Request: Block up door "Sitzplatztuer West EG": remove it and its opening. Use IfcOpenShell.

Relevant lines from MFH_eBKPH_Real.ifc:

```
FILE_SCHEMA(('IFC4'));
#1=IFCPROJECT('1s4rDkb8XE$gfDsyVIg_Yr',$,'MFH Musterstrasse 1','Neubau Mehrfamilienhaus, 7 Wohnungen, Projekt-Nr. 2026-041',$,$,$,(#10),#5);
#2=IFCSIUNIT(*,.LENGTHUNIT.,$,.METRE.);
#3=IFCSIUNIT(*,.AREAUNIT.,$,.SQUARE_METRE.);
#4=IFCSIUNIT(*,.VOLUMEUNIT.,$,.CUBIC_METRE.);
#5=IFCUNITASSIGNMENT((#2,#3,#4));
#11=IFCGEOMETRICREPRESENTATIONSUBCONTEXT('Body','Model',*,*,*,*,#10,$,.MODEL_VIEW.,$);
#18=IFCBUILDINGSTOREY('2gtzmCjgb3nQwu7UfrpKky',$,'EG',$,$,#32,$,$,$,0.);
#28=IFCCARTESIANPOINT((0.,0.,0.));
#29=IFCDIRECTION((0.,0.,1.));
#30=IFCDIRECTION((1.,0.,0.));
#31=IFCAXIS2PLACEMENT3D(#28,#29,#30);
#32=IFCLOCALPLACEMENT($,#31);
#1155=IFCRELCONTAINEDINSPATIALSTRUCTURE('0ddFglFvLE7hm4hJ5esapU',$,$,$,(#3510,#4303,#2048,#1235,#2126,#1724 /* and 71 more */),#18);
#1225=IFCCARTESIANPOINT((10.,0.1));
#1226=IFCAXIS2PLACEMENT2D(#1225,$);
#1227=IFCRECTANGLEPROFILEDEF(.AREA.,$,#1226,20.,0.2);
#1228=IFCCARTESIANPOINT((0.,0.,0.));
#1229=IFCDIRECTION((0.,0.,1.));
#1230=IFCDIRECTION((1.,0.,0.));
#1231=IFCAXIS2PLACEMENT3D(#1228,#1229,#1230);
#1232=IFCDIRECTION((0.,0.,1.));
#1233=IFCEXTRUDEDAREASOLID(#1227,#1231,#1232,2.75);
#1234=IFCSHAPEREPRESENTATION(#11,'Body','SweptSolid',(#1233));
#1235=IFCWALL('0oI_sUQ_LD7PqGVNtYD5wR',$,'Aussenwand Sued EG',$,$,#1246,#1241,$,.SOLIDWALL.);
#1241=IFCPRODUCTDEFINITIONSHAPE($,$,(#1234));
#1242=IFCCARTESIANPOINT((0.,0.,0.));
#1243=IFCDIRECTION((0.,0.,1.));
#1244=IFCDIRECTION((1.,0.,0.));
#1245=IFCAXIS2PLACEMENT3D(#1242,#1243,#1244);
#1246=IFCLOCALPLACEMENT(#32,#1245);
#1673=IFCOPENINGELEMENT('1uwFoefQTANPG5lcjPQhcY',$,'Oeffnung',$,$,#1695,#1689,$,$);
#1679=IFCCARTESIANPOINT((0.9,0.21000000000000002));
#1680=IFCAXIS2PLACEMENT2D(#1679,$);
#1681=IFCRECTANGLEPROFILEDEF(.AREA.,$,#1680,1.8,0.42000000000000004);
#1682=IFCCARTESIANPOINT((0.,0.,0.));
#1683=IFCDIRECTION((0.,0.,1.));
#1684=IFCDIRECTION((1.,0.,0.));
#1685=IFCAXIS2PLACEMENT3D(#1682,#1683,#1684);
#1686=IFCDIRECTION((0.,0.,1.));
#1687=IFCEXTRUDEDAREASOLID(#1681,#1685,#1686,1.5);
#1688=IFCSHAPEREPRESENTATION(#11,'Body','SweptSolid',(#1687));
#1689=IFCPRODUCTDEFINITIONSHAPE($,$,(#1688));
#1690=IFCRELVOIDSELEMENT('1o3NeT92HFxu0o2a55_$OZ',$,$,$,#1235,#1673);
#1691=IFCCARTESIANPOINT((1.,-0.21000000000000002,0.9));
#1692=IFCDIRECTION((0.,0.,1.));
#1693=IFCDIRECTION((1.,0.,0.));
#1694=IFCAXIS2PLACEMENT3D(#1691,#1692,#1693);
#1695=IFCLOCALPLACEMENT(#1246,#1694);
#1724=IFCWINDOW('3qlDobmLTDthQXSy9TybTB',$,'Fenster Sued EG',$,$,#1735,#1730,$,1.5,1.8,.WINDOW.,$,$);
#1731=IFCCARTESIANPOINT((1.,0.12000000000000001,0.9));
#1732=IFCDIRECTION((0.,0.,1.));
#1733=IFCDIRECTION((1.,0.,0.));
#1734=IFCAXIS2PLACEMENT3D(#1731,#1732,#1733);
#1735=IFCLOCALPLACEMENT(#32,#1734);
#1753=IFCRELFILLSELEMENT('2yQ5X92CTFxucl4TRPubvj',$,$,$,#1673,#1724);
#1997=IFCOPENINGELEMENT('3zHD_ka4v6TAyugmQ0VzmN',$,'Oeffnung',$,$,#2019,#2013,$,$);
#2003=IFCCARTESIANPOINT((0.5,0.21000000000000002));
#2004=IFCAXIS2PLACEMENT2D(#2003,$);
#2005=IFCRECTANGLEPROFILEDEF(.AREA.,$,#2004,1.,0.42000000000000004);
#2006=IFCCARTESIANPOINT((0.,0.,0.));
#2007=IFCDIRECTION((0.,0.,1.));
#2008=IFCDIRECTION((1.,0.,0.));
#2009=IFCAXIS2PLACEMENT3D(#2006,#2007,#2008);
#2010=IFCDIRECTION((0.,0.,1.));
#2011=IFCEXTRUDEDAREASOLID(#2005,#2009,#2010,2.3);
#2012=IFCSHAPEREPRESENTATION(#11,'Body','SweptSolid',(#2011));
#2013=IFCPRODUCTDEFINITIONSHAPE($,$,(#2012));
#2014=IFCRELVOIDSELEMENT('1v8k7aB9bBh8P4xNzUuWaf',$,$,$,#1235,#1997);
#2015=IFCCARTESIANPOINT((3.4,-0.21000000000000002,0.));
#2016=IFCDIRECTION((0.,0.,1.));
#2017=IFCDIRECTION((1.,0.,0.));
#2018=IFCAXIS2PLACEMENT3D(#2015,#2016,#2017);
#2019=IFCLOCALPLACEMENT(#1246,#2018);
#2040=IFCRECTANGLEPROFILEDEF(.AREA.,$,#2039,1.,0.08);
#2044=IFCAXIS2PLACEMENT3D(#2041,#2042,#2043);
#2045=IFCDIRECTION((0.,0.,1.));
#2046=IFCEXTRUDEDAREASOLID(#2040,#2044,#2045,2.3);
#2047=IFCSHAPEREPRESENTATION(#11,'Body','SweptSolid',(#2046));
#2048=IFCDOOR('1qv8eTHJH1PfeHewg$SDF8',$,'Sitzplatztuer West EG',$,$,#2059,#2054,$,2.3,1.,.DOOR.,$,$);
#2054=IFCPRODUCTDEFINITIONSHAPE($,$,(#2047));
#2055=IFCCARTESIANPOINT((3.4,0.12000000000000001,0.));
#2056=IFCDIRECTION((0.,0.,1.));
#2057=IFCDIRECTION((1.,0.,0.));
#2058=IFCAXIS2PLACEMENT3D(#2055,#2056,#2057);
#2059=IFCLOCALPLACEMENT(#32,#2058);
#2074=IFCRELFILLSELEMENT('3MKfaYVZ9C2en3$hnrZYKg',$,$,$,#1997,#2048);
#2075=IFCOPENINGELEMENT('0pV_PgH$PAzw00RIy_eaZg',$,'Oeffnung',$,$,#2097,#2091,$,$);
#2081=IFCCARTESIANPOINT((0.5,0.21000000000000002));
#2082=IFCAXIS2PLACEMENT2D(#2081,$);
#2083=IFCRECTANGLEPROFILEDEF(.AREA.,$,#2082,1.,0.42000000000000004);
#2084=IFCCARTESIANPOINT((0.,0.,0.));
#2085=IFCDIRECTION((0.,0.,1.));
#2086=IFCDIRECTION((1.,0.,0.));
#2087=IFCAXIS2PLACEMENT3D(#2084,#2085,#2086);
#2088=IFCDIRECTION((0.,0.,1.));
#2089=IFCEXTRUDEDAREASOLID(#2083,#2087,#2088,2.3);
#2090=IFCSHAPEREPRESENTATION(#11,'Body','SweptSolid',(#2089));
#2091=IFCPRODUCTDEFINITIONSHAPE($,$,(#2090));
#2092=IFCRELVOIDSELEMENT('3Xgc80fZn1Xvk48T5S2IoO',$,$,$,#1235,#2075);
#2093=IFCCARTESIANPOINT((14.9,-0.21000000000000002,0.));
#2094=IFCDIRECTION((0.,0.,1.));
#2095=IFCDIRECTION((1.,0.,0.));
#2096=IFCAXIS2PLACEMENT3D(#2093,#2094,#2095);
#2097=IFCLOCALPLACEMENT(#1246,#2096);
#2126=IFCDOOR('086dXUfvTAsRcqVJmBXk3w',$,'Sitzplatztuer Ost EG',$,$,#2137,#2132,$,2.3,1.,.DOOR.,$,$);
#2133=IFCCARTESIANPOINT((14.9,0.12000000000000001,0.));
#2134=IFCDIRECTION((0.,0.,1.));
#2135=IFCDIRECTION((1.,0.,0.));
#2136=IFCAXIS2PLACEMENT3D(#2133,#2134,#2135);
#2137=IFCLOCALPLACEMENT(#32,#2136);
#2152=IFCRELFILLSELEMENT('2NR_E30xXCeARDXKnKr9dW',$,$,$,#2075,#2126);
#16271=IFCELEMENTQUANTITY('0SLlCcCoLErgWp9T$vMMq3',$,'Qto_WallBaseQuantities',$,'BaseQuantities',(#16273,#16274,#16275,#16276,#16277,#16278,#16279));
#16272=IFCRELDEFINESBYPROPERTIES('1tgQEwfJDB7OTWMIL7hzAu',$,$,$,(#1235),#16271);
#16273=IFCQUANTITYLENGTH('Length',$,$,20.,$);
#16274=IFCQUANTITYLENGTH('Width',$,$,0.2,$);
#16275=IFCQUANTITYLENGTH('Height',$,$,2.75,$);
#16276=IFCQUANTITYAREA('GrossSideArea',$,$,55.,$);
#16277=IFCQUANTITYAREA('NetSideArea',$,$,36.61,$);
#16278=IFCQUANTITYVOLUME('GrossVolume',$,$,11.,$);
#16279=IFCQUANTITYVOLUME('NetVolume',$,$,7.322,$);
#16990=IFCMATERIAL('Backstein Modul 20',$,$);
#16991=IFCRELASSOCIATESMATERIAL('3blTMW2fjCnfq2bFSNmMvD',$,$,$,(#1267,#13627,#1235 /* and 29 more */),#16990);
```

```python
import ifcopenshell
import ifcopenshell.api.feature
import ifcopenshell.api.pset
import ifcopenshell.api.root
import ifcopenshell.geom
import ifcopenshell.util.element
import ifcopenshell.util.shape
import ifcopenshell.util.unit

model = ifcopenshell.open("MFH_eBKPH_Real.ifc")
area_scale = ifcopenshell.util.unit.calculate_unit_scale(model, "AREAUNIT")
volume_scale = ifcopenshell.util.unit.calculate_unit_scale(model, "VOLUMEUNIT")
settings = ifcopenshell.geom.settings()


def volume(element):
    """Net volume in cubic metres, openings subtracted."""
    shape = ifcopenshell.geom.create_shape(settings, element)
    return ifcopenshell.util.shape.get_volume(shape.geometry)


door = model.by_id(2048)
opening = door.FillsVoids[0].RelatingOpeningElement
wall = opening.VoidsElements[0].RelatingBuildingElement
before = volume(wall)

ifcopenshell.api.root.remove_product(model, product=door)
ifcopenshell.api.feature.remove_feature(model, feature=opening)

after = volume(wall)
thickness = 0.2  # wall thickness in metres

# Update the wall's stored quantities.
qto = model.by_id(ifcopenshell.util.element.get_pset(wall, "Qto_WallBaseQuantities", should_inherit=False)["id"])
ifcopenshell.api.pset.edit_qto(model, qto=qto, properties={
    "NetSideArea": after / thickness / area_scale,
    "NetVolume": after / volume_scale,
})

print(f"wall volume {before:.3f} -> {after:.3f} m3")

model.write("MFH_eBKPH_Real-out.ifc")
```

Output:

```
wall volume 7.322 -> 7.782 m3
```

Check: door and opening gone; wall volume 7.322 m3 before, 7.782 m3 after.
